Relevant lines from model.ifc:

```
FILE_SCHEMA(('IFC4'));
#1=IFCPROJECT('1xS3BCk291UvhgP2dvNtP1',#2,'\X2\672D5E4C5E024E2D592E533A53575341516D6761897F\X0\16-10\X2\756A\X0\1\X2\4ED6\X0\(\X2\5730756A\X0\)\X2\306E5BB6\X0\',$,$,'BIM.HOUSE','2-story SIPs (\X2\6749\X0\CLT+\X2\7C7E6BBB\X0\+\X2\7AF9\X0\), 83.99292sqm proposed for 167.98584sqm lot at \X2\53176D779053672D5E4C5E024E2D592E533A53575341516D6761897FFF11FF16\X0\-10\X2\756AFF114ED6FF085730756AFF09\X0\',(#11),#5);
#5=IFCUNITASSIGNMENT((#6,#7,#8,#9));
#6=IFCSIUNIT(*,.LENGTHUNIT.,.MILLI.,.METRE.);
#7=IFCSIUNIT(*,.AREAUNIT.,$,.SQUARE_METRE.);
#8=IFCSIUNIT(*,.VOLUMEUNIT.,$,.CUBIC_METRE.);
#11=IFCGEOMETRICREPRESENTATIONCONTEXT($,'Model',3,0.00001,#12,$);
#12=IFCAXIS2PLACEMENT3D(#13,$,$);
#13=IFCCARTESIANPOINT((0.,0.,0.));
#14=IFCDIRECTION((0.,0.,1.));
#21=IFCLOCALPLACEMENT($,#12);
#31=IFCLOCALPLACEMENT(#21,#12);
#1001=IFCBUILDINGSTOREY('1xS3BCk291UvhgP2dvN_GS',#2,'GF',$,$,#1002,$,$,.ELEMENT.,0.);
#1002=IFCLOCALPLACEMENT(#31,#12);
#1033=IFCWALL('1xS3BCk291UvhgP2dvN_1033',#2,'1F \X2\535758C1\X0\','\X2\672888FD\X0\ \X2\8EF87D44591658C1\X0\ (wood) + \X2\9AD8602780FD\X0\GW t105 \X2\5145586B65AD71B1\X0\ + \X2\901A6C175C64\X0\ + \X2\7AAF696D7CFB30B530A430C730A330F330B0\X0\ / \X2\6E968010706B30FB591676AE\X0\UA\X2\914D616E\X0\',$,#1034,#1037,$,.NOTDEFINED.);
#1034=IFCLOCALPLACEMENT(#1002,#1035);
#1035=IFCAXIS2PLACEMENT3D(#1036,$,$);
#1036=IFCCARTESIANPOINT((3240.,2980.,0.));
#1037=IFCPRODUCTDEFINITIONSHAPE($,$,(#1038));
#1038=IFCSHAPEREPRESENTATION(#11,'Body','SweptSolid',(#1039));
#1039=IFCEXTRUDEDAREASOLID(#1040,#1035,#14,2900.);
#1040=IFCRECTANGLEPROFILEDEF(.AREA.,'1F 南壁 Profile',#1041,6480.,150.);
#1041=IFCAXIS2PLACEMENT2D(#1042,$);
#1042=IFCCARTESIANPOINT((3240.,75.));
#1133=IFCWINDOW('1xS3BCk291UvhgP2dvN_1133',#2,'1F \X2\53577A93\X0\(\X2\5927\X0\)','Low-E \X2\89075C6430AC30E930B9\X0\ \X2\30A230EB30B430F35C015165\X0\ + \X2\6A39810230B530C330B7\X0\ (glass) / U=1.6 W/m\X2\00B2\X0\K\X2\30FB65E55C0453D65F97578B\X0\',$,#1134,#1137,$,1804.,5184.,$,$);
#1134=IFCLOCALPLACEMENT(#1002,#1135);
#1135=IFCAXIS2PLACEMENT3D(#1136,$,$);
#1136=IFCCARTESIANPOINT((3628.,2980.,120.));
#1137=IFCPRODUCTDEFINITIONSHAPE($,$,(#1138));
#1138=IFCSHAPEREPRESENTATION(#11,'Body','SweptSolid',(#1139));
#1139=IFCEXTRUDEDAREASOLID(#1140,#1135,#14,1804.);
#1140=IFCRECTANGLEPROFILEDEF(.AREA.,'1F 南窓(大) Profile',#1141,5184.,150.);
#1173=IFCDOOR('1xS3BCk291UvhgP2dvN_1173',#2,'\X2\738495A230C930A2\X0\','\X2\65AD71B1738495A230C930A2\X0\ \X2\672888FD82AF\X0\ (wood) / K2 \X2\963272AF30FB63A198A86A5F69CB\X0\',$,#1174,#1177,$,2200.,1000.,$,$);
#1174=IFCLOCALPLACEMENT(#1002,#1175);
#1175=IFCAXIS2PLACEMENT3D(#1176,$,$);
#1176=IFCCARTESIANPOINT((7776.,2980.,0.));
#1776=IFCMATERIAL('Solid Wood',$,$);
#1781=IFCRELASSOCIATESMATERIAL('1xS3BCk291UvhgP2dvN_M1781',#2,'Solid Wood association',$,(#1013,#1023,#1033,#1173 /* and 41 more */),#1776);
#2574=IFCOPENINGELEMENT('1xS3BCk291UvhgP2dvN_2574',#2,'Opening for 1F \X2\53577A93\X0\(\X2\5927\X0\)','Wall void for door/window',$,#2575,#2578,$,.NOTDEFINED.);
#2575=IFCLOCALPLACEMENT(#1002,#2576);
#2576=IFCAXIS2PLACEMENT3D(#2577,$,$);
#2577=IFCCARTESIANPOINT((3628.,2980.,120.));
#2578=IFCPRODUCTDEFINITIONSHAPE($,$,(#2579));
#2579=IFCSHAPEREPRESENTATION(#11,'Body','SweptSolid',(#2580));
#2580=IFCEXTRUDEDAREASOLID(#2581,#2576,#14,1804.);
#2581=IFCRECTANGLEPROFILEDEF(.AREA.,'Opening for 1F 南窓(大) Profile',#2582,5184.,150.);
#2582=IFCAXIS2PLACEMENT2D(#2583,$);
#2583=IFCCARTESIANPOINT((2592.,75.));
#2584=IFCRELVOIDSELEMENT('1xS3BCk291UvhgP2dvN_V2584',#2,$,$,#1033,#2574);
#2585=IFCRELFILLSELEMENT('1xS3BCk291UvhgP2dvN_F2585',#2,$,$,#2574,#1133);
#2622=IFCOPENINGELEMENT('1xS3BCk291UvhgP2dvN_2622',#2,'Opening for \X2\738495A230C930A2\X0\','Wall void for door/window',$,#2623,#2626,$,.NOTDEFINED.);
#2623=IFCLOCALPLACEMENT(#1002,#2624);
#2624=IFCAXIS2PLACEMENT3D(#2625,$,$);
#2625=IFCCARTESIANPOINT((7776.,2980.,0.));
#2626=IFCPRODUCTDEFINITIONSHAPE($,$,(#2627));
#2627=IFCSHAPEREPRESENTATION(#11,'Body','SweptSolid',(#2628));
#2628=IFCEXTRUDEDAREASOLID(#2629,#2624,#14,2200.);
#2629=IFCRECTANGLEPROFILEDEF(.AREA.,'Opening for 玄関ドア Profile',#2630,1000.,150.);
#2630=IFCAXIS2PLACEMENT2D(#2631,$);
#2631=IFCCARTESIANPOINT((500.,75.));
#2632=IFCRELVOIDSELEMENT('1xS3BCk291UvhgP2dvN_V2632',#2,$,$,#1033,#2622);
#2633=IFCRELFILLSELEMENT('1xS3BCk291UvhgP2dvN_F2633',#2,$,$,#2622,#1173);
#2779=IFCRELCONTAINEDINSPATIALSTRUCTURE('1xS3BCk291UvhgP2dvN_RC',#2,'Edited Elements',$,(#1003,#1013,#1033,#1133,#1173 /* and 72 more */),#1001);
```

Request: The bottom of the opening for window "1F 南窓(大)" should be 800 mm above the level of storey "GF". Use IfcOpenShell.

```python
import numpy as np
import ifcopenshell
import ifcopenshell.api.geometry
import ifcopenshell.geom
import ifcopenshell.util.element
import ifcopenshell.util.placement
import ifcopenshell.util.shape
import ifcopenshell.util.unit

model = ifcopenshell.open("model.ifc")
unit_scale = ifcopenshell.util.unit.calculate_unit_scale(model)

window = model.by_guid("1xS3BCk291UvhgP2dvN_1133")
opening = window.FillsVoids[0].RelatingOpeningElement
storey = ifcopenshell.util.element.get_container(window, ifc_class="IfcBuildingStorey")
level = ifcopenshell.util.placement.get_local_placement(storey.ObjectPlacement)[2, 3]

# The opening's origin need not be at the sill, so measure its lowest point.
shape = ifcopenshell.geom.create_shape(ifcopenshell.geom.settings(), opening)
bottom = ifcopenshell.util.shape.get_shape_bottom_elevation(shape, shape.geometry) / unit_scale
dz = level + 0.8 / unit_scale - bottom

shift = np.array([0.0, 0.0, dz])
# The window is not placed relative to its opening, so move both.
for product in (opening, window):
    matrix = ifcopenshell.util.placement.get_local_placement(product.ObjectPlacement)
    matrix[:3, 3] += shift
    ifcopenshell.api.geometry.edit_object_placement(model, product=product, matrix=matrix, is_si=False)

print(f"moved by {dz * unit_scale:+.3f} m")

model.write("model_edited.ifc")
```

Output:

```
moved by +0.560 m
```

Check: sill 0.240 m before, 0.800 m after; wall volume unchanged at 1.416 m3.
